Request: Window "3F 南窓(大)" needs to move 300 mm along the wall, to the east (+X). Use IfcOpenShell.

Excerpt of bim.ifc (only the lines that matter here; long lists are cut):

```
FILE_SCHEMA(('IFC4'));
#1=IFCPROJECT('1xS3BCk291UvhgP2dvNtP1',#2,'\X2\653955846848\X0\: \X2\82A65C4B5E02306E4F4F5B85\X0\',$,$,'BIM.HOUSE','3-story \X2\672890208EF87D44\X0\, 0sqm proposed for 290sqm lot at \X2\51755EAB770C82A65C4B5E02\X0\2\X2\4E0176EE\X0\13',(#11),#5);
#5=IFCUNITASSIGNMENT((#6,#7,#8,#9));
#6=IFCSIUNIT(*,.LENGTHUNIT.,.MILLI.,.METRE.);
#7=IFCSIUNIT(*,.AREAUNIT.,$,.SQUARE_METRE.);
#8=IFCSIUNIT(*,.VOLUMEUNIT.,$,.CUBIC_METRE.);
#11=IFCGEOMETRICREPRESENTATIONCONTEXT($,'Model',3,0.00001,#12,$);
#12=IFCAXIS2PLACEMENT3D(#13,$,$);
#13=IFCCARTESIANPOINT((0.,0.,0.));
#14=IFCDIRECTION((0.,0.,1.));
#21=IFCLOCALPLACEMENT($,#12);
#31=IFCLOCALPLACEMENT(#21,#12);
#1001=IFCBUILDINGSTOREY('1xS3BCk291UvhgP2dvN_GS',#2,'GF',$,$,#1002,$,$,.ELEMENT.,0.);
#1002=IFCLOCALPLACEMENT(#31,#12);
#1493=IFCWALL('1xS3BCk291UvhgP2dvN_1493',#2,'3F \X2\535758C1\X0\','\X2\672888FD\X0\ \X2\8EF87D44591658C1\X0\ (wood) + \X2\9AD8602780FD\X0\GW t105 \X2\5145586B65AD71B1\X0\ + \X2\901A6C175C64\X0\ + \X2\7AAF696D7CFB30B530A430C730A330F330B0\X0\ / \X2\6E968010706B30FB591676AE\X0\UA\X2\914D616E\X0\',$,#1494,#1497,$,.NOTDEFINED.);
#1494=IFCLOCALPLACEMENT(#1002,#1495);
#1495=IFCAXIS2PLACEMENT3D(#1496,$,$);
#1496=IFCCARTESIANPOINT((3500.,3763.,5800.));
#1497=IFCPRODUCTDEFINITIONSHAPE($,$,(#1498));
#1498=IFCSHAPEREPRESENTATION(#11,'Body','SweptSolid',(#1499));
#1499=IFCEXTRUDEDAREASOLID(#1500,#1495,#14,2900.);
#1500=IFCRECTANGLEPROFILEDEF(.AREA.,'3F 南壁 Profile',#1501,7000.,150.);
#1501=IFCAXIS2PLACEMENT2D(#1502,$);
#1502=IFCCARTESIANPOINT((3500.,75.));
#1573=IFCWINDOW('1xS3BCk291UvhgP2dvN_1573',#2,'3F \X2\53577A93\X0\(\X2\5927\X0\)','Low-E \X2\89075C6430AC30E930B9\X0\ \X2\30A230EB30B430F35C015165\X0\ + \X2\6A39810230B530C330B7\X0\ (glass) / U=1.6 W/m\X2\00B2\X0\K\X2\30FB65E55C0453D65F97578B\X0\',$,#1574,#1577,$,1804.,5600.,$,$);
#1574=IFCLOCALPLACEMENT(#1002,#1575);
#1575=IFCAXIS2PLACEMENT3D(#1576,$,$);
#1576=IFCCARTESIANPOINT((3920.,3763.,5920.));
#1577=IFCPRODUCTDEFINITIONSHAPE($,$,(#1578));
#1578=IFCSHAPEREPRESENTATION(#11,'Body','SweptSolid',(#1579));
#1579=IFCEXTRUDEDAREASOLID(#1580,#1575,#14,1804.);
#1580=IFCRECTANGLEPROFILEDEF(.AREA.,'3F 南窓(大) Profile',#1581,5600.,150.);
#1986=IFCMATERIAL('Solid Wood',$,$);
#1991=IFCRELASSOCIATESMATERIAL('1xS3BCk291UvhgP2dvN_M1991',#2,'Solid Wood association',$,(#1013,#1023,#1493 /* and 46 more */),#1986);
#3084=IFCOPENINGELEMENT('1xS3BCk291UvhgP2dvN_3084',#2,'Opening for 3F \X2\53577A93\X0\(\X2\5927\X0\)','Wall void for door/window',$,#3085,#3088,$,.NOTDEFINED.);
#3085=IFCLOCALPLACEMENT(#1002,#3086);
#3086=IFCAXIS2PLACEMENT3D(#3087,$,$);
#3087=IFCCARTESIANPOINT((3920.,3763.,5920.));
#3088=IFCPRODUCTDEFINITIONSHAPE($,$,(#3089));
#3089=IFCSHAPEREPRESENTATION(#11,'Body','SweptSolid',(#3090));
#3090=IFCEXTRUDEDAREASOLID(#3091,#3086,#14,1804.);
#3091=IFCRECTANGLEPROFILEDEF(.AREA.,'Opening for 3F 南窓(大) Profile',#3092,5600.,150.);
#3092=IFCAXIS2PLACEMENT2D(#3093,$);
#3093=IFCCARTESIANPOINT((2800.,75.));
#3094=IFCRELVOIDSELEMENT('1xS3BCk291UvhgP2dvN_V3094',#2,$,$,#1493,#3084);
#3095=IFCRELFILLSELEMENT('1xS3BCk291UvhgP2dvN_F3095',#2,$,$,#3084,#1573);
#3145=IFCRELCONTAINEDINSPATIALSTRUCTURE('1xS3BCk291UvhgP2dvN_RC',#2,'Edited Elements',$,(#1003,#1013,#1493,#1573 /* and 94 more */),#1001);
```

```python
import ifcopenshell
import ifcopenshell.api.geometry
import ifcopenshell.util.placement
import ifcopenshell.util.unit

model = ifcopenshell.open("bim.ifc")
unit_scale = ifcopenshell.util.unit.calculate_unit_scale(model)

window = model.by_guid("1xS3BCk291UvhgP2dvN_1573")
opening = window.FillsVoids[0].RelatingOpeningElement
wall = opening.VoidsElements[0].RelatingBuildingElement

wall_matrix = ifcopenshell.util.placement.get_local_placement(wall.ObjectPlacement)
shift = wall_matrix[:3, 0] * 0.3 / unit_scale
before = ifcopenshell.util.placement.get_local_placement(window.ObjectPlacement)[:3, 3].copy()

# The window is not placed relative to its opening, so move both.
for product in (opening, window):
    matrix = ifcopenshell.util.placement.get_local_placement(product.ObjectPlacement)
    matrix[:3, 3] += shift
    ifcopenshell.api.geometry.edit_object_placement(model, product=product, matrix=matrix, is_si=False)

after = ifcopenshell.util.placement.get_local_placement(window.ObjectPlacement)[:3, 3]
print("window moved by", (after - before).round(3) + 0.0)

model.write("bim_updated.ifc")
```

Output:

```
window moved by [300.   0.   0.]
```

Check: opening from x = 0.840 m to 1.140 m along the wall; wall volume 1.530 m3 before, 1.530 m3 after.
